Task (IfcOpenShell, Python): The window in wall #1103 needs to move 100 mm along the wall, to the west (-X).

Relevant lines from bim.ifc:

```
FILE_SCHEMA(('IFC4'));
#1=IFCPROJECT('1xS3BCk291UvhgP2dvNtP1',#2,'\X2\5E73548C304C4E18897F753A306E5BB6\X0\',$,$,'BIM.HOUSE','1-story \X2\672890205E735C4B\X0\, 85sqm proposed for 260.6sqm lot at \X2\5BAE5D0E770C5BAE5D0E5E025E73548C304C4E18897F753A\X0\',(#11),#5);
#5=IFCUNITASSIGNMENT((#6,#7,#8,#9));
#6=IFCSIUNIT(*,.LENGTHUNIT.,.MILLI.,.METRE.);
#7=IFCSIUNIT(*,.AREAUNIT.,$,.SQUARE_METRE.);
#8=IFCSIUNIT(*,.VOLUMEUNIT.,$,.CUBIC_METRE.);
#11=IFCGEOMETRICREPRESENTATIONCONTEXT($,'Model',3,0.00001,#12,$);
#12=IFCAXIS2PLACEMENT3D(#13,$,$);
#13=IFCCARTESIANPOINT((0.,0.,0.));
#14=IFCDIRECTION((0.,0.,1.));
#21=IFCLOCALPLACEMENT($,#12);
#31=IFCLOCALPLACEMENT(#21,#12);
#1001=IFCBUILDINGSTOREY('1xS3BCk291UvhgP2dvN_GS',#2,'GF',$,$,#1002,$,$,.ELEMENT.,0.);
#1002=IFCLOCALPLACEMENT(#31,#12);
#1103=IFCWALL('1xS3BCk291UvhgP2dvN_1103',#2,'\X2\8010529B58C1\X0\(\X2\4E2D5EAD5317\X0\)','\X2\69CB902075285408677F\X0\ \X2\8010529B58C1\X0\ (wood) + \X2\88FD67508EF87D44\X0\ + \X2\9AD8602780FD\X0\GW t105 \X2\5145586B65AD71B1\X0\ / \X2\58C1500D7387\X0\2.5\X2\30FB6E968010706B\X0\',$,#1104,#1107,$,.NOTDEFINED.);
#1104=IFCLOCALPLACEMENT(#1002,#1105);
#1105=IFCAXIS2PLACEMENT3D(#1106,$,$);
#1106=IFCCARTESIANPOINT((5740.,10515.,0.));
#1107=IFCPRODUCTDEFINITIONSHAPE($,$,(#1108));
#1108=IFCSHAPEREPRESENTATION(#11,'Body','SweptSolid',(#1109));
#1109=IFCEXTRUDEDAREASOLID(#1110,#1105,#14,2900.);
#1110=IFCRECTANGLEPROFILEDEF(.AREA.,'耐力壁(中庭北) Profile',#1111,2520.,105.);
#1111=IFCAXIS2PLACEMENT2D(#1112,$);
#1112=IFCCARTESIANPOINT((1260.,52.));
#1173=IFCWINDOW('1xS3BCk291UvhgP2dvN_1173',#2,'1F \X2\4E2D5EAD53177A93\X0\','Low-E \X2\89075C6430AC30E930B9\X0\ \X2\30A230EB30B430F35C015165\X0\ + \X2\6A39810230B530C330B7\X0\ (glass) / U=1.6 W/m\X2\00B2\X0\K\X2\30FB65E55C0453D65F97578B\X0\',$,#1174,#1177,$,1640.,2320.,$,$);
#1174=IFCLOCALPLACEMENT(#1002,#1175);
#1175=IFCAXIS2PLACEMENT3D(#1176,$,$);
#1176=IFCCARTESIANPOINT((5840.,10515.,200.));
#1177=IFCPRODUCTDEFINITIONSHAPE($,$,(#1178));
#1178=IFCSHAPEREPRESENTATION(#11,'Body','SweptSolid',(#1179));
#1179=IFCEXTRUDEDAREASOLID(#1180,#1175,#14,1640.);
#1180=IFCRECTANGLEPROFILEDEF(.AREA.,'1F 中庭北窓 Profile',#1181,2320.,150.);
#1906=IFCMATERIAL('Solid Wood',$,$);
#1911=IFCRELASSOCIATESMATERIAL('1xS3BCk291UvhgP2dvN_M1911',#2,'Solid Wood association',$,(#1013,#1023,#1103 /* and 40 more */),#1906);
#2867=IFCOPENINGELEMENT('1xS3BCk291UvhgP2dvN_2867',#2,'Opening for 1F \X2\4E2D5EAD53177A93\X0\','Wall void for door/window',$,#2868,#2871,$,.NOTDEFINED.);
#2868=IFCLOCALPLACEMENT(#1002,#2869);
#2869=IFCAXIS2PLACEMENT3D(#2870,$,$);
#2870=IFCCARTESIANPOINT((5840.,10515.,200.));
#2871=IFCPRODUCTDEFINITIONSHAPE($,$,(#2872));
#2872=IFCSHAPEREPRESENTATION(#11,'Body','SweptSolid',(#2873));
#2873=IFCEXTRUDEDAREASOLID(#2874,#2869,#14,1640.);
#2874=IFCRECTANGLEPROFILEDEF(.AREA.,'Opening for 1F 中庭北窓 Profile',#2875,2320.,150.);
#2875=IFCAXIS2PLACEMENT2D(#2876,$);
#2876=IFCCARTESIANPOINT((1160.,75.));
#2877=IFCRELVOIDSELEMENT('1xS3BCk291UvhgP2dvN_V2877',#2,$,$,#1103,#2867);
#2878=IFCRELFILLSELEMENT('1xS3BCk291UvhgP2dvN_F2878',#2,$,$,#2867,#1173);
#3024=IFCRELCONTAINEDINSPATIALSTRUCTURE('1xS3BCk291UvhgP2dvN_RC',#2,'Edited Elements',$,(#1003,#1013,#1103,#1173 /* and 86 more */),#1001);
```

```python
import ifcopenshell
import ifcopenshell.api.geometry
import ifcopenshell.util.placement
import ifcopenshell.util.unit

model = ifcopenshell.open("bim.ifc")
unit_scale = ifcopenshell.util.unit.calculate_unit_scale(model)

window = model.by_id(1173)
opening = window.FillsVoids[0].RelatingOpeningElement
wall = opening.VoidsElements[0].RelatingBuildingElement

wall_matrix = ifcopenshell.util.placement.get_local_placement(wall.ObjectPlacement)
shift = wall_matrix[:3, 0] * -0.1 / unit_scale
before = ifcopenshell.util.placement.get_local_placement(window.ObjectPlacement)[:3, 3].copy()

# The window is not placed relative to its opening, so move both.
for product in (opening, window):
    matrix = ifcopenshell.util.placement.get_local_placement(product.ObjectPlacement)
    matrix[:3, 3] += shift
    ifcopenshell.api.geometry.edit_object_placement(model, product=product, matrix=matrix, is_si=False)

after = ifcopenshell.util.placement.get_local_placement(window.ObjectPlacement)[:3, 3]
print("window moved by", (after - before).round(3) + 0.0)

model.write("bim-out.ifc")
```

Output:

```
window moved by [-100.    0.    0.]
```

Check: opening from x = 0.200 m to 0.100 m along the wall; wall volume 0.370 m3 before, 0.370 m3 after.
